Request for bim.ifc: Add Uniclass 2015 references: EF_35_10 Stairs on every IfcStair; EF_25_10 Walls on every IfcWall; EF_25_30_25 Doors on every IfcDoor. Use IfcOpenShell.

First a look at what the model holds.

```python
import ifcopenshell

model = ifcopenshell.open("bim.ifc")
print(model.schema)
print("classifications:", [c.Name for c in model.by_type("IfcClassification")])
for ifc_class in ("IfcDoor", "IfcRoof", "IfcStair", "IfcWall", "IfcWindow"):
    print(ifc_class, len(model.by_type(ifc_class)))
```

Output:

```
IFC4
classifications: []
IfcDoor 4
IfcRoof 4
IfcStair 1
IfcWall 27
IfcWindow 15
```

```python
import ifcopenshell
import ifcopenshell.api.classification

model = ifcopenshell.open("bim.ifc")

system = ifcopenshell.api.classification.add_classification(model, classification="Uniclass 2015")

codes = {
    "IfcStair": ("EF_35_10", "Stairs"),
    "IfcWall": ("EF_25_10", "Walls"),
    "IfcDoor": ("EF_25_30_25", "Doors"),
}
for ifc_class, (code, name) in codes.items():
    products = model.by_type(ifc_class)
    ifcopenshell.api.classification.add_reference(
        model, products=products, classification=system, identification=code, name=name
    )
    print(code, len(products))

model.write("bim_updated.ifc")
```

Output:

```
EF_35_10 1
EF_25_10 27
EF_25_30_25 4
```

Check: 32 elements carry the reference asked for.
